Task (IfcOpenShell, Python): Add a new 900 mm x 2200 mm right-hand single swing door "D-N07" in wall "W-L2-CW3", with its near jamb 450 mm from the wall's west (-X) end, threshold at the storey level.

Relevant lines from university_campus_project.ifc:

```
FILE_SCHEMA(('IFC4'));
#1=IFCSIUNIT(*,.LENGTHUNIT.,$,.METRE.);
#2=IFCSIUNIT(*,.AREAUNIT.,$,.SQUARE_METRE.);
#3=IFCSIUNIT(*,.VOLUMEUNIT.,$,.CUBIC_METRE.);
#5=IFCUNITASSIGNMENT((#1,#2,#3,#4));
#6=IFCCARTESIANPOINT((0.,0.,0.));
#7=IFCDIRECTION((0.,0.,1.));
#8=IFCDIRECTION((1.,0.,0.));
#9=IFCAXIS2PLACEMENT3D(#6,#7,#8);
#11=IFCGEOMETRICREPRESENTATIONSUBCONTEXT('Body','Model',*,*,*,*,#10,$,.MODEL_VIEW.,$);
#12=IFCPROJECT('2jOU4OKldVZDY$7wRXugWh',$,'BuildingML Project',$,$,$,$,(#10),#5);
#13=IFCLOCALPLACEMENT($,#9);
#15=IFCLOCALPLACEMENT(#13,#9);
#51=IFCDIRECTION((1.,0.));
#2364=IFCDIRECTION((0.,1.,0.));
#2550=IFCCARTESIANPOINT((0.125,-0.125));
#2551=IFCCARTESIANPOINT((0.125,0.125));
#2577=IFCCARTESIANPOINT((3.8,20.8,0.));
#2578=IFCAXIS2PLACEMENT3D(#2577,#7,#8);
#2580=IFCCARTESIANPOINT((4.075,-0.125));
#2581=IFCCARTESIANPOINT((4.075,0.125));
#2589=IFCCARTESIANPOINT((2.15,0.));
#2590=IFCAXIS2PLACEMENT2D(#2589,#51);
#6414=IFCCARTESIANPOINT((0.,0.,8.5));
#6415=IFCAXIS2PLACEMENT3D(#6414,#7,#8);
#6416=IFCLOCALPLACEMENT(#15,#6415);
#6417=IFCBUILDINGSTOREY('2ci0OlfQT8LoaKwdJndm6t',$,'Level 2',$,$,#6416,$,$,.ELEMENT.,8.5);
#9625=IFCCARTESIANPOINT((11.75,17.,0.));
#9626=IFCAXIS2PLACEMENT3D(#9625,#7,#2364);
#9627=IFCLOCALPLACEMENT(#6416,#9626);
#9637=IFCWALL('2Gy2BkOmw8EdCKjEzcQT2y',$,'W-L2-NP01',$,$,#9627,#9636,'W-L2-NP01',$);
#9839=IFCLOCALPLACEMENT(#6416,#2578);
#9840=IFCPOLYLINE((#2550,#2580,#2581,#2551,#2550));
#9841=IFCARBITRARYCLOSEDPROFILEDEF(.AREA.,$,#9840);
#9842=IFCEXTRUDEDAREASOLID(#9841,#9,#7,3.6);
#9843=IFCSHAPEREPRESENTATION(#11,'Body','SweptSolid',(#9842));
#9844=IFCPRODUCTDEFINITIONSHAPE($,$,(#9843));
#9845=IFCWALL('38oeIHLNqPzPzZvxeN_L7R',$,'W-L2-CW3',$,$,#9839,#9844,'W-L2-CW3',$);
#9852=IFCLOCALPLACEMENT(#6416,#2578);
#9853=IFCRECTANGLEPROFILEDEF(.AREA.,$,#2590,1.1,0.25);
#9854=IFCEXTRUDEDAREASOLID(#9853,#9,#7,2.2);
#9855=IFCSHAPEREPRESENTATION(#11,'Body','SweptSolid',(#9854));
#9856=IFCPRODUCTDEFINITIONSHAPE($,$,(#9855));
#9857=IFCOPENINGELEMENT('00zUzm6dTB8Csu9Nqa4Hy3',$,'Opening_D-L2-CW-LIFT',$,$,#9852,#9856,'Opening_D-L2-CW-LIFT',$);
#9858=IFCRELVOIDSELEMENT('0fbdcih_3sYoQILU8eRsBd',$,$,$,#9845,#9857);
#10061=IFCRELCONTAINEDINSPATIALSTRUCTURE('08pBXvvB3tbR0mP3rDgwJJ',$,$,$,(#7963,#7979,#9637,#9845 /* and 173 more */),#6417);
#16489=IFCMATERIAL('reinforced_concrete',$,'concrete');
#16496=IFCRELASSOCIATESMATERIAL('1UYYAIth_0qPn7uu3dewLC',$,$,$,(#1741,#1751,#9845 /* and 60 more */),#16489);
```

```python
import numpy as np
import ifcopenshell
import ifcopenshell.api.feature
import ifcopenshell.api.geometry
import ifcopenshell.api.root
import ifcopenshell.api.spatial
import ifcopenshell.geom
import ifcopenshell.util.element
import ifcopenshell.util.placement
import ifcopenshell.util.representation
import ifcopenshell.util.shape
import ifcopenshell.util.unit

model = ifcopenshell.open("university_campus_project.ifc")
unit_scale = ifcopenshell.util.unit.calculate_unit_scale(model)
settings = ifcopenshell.geom.settings()


def volume(element):
    """Net volume in cubic metres, openings subtracted."""
    shape = ifcopenshell.geom.create_shape(settings, element)
    return ifcopenshell.util.shape.get_volume(shape.geometry)


wall = model.by_id(9845)
storey = ifcopenshell.util.element.get_container(wall, ifc_class="IfcBuildingStorey")
context = ifcopenshell.util.representation.get_context(model, "Model", "Body", "MODEL_VIEW")
before = volume(wall)

width, height, from_end, sill = 0.9, 2.2, 0.45, 0.0  # metres

# The wall runs along its own X axis, and the end named is its -X end.
wall_shape = ifcopenshell.geom.create_shape(settings, wall)
x, y, z = ifcopenshell.util.shape.get_vertices(wall_shape.geometry).T
start = x.min() + from_end
face, thickness = float(y.min()), float(y.max() - y.min())
wall_matrix = ifcopenshell.util.placement.get_local_placement(wall.ObjectPlacement)
level = ifcopenshell.util.placement.get_local_placement(storey.ObjectPlacement)[2, 3]


def in_wall(x, y):
    """Placement at x, y metres in the wall's axes, at sill height."""
    matrix = wall_matrix.copy()
    matrix[:, 3] = wall_matrix @ np.array([x / unit_scale, y / unit_scale, 0.0, 1.0])
    matrix[2, 3] = level + sill / unit_scale
    return matrix


# Opening: a box that overshoots both wall faces by 50 mm.
opening = ifcopenshell.api.root.create_entity(model, ifc_class="IfcOpeningElement", predefined_type="OPENING")
box = ifcopenshell.api.geometry.add_wall_representation(
    model, context=context, length=width, height=height, thickness=thickness + 0.1
)
ifcopenshell.api.geometry.assign_representation(model, product=opening, representation=box)
ifcopenshell.api.geometry.edit_object_placement(model, product=opening, matrix=in_wall(start, face - 0.05), is_si=False)
ifcopenshell.api.feature.add_feature(model, feature=opening, element=wall)

door = ifcopenshell.api.root.create_entity(model, ifc_class="IfcDoor", name="D-N07", predefined_type="DOOR")
door.OverallWidth, door.OverallHeight = width / unit_scale, height / unit_scale
door.OperationType = "SINGLE_SWING_RIGHT"
body = ifcopenshell.api.geometry.add_door_representation(
    model,
    context=context,
    overall_width=door.OverallWidth,
    overall_height=door.OverallHeight,
    operation_type="SINGLE_SWING_RIGHT",
    lining_properties={"LiningDepth": thickness / unit_scale, "ThresholdDepth": thickness / unit_scale},
)
ifcopenshell.api.geometry.assign_representation(model, product=door, representation=body)
ifcopenshell.api.spatial.assign_container(model, products=[door], relating_structure=storey)
ifcopenshell.api.feature.add_filling(model, opening=opening, element=door)

# The lining spans the wall, so the door starts at the wall face.
ifcopenshell.api.geometry.edit_object_placement(model, product=door, matrix=in_wall(start, face), is_si=False)

after = volume(wall)

print(f"wall volume {before:.3f} -> {after:.3f} m3")

model.write("university_campus_project_v2.ifc")
```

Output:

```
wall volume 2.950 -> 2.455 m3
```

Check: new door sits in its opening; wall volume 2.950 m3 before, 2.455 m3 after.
